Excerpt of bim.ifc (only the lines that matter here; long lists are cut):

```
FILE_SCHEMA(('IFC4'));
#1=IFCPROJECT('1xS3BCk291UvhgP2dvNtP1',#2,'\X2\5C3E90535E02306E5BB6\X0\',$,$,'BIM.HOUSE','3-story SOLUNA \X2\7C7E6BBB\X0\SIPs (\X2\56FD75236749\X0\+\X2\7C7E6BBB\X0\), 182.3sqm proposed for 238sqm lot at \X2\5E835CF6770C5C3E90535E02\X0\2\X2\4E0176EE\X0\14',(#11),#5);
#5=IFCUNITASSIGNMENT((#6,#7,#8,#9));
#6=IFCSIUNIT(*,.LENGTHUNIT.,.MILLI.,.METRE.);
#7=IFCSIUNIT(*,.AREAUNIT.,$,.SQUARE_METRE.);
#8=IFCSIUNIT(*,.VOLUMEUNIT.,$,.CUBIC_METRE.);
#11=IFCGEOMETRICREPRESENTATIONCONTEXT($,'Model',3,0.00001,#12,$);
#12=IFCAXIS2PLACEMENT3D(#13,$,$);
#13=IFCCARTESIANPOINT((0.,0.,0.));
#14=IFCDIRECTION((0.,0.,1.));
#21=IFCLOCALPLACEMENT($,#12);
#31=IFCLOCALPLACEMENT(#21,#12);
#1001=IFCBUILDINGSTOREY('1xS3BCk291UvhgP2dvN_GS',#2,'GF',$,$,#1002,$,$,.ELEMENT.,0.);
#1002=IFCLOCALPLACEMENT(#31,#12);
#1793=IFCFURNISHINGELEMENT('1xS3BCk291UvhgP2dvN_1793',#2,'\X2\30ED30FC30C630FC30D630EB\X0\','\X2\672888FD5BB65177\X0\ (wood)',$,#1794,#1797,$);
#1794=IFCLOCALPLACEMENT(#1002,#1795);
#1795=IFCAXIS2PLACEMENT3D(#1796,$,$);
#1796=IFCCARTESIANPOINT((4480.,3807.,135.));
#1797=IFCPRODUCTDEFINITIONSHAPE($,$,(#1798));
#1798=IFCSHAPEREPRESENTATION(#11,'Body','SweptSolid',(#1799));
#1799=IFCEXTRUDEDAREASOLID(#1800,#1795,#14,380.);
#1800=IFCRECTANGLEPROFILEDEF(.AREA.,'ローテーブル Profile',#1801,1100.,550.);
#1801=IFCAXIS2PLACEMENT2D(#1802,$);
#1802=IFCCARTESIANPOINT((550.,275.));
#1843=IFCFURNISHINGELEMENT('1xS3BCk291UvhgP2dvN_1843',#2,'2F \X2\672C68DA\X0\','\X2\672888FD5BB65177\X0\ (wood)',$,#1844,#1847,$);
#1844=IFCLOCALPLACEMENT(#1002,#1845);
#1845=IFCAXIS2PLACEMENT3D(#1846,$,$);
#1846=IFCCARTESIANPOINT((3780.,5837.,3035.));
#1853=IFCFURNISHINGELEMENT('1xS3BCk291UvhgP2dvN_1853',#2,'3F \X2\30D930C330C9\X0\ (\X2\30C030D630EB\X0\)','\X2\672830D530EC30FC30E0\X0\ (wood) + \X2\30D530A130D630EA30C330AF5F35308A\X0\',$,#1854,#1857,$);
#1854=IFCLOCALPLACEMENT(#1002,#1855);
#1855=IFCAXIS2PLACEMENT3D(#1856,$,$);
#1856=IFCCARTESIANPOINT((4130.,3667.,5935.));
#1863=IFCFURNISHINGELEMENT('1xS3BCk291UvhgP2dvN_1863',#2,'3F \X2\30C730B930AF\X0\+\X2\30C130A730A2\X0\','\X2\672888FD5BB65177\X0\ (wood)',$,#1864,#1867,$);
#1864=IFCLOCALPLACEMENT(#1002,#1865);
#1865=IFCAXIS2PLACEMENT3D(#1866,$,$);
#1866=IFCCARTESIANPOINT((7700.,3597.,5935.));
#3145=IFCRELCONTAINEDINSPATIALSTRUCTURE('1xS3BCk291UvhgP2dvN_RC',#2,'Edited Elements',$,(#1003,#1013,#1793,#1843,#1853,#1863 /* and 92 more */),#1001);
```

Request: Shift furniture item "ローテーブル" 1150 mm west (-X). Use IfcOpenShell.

```python
import ifcopenshell
import ifcopenshell.api.geometry
import ifcopenshell.util.placement

model = ifcopenshell.open("bim.ifc")

item = model.by_guid("1xS3BCk291UvhgP2dvN_1793")
matrix = ifcopenshell.util.placement.get_local_placement(item.ObjectPlacement)
matrix[0, 3] -= 1150.0
ifcopenshell.api.geometry.edit_object_placement(model, product=item, matrix=matrix, is_si=False)

print(ifcopenshell.util.placement.get_local_placement(item.ObjectPlacement).round(3) + 0.0)

model.write("bim_updated.ifc")
```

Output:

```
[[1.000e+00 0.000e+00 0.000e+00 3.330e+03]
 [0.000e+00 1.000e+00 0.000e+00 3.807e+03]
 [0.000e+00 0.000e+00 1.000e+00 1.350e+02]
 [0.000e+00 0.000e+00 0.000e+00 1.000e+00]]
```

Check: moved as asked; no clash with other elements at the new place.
